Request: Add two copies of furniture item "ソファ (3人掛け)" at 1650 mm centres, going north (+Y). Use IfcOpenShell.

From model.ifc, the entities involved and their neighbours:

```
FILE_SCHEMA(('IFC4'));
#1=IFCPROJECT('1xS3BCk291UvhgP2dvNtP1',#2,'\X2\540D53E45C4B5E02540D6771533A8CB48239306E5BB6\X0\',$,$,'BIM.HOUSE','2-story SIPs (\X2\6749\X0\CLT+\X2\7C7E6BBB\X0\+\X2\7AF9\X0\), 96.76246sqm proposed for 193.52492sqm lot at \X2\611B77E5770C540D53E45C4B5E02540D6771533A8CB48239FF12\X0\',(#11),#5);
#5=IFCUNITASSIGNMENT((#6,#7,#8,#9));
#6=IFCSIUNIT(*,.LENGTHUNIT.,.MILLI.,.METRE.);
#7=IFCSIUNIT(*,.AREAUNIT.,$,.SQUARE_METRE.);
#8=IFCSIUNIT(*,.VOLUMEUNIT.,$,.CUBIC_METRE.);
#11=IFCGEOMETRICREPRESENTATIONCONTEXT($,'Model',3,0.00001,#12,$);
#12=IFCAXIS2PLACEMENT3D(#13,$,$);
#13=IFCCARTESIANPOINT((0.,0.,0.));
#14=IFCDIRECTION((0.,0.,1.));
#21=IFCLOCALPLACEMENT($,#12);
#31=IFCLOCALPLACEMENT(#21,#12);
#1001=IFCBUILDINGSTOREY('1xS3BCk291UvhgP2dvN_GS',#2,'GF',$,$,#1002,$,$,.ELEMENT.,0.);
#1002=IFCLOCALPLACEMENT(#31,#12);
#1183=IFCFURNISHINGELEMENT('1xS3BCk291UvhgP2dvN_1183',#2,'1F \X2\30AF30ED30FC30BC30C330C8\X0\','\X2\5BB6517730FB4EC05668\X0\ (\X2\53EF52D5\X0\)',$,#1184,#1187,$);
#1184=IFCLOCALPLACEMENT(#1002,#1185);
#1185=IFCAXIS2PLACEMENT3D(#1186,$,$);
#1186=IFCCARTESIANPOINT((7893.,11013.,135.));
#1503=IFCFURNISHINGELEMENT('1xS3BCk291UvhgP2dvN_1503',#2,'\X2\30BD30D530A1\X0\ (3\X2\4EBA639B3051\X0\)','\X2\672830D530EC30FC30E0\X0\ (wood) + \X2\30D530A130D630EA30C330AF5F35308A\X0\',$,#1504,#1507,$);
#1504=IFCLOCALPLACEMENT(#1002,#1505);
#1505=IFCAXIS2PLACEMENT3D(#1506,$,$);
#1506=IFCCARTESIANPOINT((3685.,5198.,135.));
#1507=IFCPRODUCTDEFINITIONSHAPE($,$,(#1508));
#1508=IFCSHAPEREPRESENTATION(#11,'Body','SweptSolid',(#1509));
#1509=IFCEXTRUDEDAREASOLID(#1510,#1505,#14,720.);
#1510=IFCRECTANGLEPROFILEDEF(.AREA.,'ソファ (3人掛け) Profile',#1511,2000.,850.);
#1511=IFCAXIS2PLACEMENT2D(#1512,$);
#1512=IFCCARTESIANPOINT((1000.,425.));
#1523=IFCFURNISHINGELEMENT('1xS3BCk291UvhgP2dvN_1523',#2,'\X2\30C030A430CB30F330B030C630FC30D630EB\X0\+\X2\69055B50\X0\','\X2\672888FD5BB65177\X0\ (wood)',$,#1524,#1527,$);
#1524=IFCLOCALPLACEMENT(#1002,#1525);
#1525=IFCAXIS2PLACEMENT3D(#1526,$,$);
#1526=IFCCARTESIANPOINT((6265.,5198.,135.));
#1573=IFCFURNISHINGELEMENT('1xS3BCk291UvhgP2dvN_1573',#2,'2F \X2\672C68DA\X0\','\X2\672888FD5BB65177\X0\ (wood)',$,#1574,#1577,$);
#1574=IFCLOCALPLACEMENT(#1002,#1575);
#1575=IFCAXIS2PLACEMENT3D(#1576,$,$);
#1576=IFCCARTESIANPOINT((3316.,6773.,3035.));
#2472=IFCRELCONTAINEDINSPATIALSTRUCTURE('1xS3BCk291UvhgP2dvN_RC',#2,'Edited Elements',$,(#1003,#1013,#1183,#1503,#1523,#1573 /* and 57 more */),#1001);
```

```python
import numpy as np
import ifcopenshell
import ifcopenshell.api.geometry
import ifcopenshell.api.root
import ifcopenshell.util.element
import ifcopenshell.util.placement

model = ifcopenshell.open("model.ifc")


def reuse_history(source, copy):
    """copy_class also copies each property set's owner history, people and application; keep the originals."""
    for rel in copy.IsDefinedBy:
        if rel.is_a("IfcRelDefinesByProperties") and (history := rel.RelatingPropertyDefinition.OwnerHistory):
            rel.RelatingPropertyDefinition.OwnerHistory = source.OwnerHistory
            ifcopenshell.util.element.remove_deep2(model, history)


source = model.by_id(1503)
base = ifcopenshell.util.placement.get_local_placement(source.ObjectPlacement)
step = np.array([0.0, 1.0, 0.0]) * 1650.0

for i in range(1, 3):
    copy = ifcopenshell.api.root.copy_class(model, product=source)
    copy.Representation = ifcopenshell.util.element.copy_deep(
        model, source.Representation, exclude=["IfcGeometricRepresentationContext", "IfcRepresentationMap"]
    )
    reuse_history(source, copy)
    matrix = base.copy()
    matrix[:3, 3] += i * step
    print("added at", matrix[:3, 3].round(3) + 0.0)
    ifcopenshell.api.geometry.edit_object_placement(model, product=copy, matrix=matrix, is_si=False)

model.write("model_edited.ifc")
```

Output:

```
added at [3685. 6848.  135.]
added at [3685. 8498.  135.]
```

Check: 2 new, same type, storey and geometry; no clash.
